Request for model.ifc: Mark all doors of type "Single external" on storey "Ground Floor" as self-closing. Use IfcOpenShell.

First a look at what the model holds.

```python
import ifcopenshell
import ifcopenshell.util.element

model = ifcopenshell.open("model.ifc")
print(model.schema)
storey = next(s for s in model.by_type("IfcBuildingStorey") if s.Name == "Ground Floor")
doors = [e for e in ifcopenshell.util.element.get_decomposition(storey) if e.is_a("IfcDoor")]
seen = {}
for e in doors:
    element_type = ifcopenshell.util.element.get_type(e)
    key = (element_type.Name if element_type != e and element_type else None, ifcopenshell.util.element.get_pset(e, "Pset_DoorCommon", "SelfClosing"))
    seen[key] = seen.get(key, 0) + 1
for (name, value), count in sorted(seen.items(), key=str):
    print(count, "x", name, "|", value)
```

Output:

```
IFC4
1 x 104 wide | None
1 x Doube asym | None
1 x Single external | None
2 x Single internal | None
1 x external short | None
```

```python
import ifcopenshell
import ifcopenshell.api.pset
import ifcopenshell.util.element

model = ifcopenshell.open("model.ifc")

storey = next(s for s in model.by_type("IfcBuildingStorey") if s.Name == "Ground Floor")
doors = [e for e in ifcopenshell.util.element.get_decomposition(storey) if e.is_a("IfcDoor")]

count = 0
for e in doors:
    element_type = ifcopenshell.util.element.get_type(e)
    if element_type in (None, e) or element_type.Name != "Single external":
        continue
    # add_pset returns the element's existing set when there is one.
    pset = ifcopenshell.api.pset.add_pset(model, product=e, name="Pset_DoorCommon")
    ifcopenshell.api.pset.edit_pset(model, pset=pset, properties={"SelfClosing": True})
    count += 1

print(count, "doors updated")

model.write("model_rev.ifc")
```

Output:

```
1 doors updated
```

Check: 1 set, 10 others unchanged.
